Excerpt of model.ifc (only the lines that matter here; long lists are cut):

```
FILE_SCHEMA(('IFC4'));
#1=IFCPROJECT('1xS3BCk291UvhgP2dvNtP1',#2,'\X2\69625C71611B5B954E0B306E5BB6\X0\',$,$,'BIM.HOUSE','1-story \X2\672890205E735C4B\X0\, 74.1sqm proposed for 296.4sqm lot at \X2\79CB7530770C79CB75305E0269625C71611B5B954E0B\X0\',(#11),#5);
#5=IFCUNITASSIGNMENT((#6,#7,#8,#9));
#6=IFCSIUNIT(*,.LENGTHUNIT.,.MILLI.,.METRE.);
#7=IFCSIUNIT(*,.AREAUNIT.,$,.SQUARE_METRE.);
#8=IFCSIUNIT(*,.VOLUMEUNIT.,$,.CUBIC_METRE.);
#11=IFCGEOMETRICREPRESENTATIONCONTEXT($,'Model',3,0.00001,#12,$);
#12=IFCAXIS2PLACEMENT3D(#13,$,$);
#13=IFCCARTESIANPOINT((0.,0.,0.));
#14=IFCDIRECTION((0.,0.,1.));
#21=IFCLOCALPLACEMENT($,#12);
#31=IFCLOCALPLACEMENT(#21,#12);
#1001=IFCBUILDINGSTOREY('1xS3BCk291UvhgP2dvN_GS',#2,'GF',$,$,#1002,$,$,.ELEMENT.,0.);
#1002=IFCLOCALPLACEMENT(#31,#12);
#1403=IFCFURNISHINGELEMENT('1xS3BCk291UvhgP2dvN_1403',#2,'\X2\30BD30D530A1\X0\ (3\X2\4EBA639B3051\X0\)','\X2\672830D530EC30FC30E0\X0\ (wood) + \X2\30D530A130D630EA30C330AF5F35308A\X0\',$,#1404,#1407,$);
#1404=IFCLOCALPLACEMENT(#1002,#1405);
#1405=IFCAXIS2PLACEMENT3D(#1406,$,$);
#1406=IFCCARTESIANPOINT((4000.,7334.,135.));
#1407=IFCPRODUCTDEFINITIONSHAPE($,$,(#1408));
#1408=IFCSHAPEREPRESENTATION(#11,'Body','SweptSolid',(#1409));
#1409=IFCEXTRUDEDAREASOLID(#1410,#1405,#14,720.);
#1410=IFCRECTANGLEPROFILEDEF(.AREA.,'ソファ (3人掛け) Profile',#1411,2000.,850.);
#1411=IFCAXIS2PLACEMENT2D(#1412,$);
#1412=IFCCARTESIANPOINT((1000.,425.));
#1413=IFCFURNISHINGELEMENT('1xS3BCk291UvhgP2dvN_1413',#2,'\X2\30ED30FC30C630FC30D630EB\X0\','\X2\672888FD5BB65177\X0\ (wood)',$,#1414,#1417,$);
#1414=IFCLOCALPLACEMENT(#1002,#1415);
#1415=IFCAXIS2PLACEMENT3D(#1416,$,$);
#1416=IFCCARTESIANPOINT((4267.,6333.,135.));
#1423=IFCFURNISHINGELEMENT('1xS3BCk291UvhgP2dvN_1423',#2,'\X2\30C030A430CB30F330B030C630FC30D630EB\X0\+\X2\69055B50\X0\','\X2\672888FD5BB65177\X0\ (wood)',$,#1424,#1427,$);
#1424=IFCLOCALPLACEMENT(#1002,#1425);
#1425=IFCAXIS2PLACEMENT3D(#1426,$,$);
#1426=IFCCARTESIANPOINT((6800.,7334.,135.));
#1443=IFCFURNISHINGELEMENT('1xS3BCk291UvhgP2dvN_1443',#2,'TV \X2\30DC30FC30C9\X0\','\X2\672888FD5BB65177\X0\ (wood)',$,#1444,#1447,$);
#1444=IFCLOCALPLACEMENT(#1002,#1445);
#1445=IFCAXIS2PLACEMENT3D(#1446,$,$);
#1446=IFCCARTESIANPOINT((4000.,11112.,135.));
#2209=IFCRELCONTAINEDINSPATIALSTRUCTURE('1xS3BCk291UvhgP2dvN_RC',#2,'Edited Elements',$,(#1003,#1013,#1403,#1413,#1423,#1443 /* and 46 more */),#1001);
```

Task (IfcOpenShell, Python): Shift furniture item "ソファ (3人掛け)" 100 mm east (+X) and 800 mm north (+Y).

```python
import ifcopenshell
import ifcopenshell.api.geometry
import ifcopenshell.util.placement

model = ifcopenshell.open("model.ifc")

item = model.by_guid("1xS3BCk291UvhgP2dvN_1403")
matrix = ifcopenshell.util.placement.get_local_placement(item.ObjectPlacement)
matrix[0, 3] += 100.0
matrix[1, 3] += 800.0
ifcopenshell.api.geometry.edit_object_placement(model, product=item, matrix=matrix, is_si=False)

print(ifcopenshell.util.placement.get_local_placement(item.ObjectPlacement).round(3) + 0.0)

model.write("model_rev.ifc")
```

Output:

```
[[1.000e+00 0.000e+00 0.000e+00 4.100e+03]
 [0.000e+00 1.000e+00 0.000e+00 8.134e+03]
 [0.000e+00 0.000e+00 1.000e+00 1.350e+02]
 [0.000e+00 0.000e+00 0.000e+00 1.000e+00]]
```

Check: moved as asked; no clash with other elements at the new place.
